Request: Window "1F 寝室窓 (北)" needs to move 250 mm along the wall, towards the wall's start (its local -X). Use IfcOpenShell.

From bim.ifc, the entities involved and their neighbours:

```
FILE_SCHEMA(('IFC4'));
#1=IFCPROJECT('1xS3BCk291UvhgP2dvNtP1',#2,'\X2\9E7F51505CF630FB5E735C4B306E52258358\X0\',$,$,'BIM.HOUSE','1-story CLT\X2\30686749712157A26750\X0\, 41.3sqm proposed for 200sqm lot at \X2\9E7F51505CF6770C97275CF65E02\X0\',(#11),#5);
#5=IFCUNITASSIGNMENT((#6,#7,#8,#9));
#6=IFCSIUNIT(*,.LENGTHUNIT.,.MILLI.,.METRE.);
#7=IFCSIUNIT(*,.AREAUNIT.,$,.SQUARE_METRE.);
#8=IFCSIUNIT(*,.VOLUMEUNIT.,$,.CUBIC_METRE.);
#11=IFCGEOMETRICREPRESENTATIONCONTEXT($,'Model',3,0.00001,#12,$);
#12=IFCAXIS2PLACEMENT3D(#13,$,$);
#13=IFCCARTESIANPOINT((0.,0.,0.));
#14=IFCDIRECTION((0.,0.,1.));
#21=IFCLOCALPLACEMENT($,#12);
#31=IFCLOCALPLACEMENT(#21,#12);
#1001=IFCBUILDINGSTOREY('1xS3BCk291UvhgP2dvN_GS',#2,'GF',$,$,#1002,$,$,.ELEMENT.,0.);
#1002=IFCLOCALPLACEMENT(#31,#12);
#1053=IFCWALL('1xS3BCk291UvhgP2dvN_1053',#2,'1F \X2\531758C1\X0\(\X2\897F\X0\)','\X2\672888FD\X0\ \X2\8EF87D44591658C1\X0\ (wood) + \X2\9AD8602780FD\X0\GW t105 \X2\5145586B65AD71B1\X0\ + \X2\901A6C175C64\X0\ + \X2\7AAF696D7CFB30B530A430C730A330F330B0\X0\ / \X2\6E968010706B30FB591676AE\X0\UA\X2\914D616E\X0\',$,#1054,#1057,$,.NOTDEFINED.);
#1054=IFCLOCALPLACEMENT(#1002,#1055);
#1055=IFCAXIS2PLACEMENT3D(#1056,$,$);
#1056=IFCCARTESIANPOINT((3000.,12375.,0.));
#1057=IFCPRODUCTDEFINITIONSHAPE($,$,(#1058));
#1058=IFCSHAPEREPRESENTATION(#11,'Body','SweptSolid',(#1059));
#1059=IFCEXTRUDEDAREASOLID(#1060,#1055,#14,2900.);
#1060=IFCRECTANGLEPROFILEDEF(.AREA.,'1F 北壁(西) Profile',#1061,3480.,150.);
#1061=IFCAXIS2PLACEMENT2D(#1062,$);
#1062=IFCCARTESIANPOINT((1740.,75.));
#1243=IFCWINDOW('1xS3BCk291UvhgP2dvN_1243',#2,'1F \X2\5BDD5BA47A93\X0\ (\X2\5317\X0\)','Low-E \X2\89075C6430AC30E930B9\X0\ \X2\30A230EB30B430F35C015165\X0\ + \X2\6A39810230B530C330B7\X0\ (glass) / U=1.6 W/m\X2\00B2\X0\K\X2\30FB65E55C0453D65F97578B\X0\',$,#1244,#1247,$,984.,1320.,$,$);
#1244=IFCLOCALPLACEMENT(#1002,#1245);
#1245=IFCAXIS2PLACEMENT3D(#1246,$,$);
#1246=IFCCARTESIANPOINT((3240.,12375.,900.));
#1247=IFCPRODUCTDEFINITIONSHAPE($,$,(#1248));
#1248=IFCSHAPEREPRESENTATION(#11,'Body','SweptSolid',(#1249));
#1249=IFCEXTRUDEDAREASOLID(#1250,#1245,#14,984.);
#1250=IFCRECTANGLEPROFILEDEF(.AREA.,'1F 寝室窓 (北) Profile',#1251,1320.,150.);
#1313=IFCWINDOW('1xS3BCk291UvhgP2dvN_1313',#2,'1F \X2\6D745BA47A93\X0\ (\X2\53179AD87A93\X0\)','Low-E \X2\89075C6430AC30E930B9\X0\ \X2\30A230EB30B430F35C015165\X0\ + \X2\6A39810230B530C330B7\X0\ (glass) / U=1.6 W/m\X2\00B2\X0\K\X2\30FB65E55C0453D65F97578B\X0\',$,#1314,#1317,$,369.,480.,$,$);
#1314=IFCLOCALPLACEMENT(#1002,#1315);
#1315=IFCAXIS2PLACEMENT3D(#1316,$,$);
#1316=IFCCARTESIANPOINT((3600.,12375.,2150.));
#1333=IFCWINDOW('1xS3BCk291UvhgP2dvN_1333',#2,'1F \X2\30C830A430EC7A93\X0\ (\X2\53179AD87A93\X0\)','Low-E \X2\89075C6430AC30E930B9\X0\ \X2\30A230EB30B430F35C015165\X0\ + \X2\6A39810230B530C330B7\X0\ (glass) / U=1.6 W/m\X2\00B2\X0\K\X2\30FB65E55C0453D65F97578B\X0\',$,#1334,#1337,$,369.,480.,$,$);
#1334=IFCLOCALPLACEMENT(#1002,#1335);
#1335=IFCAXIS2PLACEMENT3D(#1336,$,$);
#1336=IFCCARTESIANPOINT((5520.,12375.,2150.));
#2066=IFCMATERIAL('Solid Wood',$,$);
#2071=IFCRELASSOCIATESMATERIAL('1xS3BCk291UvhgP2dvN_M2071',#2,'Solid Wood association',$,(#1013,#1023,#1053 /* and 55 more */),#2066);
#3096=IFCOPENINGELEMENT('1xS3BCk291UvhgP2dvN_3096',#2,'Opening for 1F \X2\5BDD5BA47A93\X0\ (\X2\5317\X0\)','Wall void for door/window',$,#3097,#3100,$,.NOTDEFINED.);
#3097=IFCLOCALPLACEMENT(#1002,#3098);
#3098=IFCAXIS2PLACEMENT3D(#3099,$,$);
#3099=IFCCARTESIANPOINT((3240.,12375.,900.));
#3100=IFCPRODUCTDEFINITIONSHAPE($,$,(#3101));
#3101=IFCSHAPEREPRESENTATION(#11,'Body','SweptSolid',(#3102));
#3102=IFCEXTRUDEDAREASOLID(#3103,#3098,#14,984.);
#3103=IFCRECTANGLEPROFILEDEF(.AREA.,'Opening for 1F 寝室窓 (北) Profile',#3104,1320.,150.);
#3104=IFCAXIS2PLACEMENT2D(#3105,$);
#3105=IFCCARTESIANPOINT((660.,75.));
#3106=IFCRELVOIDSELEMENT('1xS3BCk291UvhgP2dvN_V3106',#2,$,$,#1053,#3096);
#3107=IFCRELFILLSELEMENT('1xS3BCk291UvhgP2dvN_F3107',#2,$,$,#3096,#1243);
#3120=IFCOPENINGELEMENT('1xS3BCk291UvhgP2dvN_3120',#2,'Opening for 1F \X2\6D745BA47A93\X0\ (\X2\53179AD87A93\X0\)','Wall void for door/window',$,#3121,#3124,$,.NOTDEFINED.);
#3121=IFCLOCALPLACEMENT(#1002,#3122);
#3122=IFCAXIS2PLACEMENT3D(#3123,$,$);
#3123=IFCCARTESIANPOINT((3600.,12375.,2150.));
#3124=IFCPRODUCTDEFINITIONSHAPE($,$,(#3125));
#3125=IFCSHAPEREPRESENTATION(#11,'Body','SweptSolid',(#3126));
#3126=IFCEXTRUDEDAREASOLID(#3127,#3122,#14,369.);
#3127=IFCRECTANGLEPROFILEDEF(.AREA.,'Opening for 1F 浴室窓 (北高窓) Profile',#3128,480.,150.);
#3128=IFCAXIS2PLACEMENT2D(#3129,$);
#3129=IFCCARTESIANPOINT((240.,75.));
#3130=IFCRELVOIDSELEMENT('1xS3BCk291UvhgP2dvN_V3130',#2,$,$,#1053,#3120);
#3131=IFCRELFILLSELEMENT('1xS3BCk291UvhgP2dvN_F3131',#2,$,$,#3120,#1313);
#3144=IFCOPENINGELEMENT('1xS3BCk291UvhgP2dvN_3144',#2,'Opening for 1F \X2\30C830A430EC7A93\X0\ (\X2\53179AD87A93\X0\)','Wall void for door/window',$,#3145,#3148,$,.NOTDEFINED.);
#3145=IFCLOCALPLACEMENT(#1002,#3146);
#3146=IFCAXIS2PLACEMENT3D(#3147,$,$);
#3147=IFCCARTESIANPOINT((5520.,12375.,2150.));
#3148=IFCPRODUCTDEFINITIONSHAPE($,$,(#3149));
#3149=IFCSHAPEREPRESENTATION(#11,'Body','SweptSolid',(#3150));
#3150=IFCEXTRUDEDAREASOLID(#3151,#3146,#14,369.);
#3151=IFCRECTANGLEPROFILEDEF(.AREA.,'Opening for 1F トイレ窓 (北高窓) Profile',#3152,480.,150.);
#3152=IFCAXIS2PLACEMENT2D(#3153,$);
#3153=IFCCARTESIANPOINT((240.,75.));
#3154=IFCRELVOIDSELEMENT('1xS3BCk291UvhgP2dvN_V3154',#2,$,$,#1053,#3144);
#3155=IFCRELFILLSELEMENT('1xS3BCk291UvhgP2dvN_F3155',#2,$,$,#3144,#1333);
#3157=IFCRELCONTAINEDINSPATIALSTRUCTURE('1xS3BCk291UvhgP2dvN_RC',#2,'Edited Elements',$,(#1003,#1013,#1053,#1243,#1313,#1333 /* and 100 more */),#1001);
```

```python
import ifcopenshell
import ifcopenshell.api.geometry
import ifcopenshell.util.placement

model = ifcopenshell.open("bim.ifc")

window = model.by_guid("1xS3BCk291UvhgP2dvN_1243")
opening = window.FillsVoids[0].RelatingOpeningElement
wall = opening.VoidsElements[0].RelatingBuildingElement

wall_matrix = ifcopenshell.util.placement.get_local_placement(wall.ObjectPlacement)
shift = wall_matrix[:3, 0] * -250.0
before = ifcopenshell.util.placement.get_local_placement(window.ObjectPlacement)[:3, 3].copy()

# The window is not placed relative to its opening, so move both.
for product in (opening, window):
    matrix = ifcopenshell.util.placement.get_local_placement(product.ObjectPlacement)
    matrix[:3, 3] += shift
    ifcopenshell.api.geometry.edit_object_placement(model, product=product, matrix=matrix, is_si=False)

after = ifcopenshell.util.placement.get_local_placement(window.ObjectPlacement)[:3, 3]
print("window moved by", (after - before).round(3) + 0.0)

model.write("bim_v2.ifc")
```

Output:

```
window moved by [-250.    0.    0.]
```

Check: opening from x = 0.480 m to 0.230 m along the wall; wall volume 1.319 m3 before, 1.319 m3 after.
